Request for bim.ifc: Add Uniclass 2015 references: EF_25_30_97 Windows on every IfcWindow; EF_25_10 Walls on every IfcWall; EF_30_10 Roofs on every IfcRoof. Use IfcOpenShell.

First a look at what the model holds.

```python
import ifcopenshell

model = ifcopenshell.open("bim.ifc")
print(model.schema)
print("classifications:", [c.Name for c in model.by_type("IfcClassification")])
for ifc_class in ("IfcDoor", "IfcRoof", "IfcStair", "IfcWall", "IfcWindow"):
    print(ifc_class, len(model.by_type(ifc_class)))
```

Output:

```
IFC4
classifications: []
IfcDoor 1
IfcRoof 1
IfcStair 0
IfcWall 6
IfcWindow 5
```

```python
import ifcopenshell
import ifcopenshell.api.classification

model = ifcopenshell.open("bim.ifc")

system = ifcopenshell.api.classification.add_classification(model, classification="Uniclass 2015")

codes = {
    "IfcWindow": ("EF_25_30_97", "Windows"),
    "IfcWall": ("EF_25_10", "Walls"),
    "IfcRoof": ("EF_30_10", "Roofs"),
}
for ifc_class, (code, name) in codes.items():
    products = model.by_type(ifc_class)
    ifcopenshell.api.classification.add_reference(
        model, products=products, classification=system, identification=code, name=name
    )
    print(code, len(products))

model.write("bim_edited.ifc")
```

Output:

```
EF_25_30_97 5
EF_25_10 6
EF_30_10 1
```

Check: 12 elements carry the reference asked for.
